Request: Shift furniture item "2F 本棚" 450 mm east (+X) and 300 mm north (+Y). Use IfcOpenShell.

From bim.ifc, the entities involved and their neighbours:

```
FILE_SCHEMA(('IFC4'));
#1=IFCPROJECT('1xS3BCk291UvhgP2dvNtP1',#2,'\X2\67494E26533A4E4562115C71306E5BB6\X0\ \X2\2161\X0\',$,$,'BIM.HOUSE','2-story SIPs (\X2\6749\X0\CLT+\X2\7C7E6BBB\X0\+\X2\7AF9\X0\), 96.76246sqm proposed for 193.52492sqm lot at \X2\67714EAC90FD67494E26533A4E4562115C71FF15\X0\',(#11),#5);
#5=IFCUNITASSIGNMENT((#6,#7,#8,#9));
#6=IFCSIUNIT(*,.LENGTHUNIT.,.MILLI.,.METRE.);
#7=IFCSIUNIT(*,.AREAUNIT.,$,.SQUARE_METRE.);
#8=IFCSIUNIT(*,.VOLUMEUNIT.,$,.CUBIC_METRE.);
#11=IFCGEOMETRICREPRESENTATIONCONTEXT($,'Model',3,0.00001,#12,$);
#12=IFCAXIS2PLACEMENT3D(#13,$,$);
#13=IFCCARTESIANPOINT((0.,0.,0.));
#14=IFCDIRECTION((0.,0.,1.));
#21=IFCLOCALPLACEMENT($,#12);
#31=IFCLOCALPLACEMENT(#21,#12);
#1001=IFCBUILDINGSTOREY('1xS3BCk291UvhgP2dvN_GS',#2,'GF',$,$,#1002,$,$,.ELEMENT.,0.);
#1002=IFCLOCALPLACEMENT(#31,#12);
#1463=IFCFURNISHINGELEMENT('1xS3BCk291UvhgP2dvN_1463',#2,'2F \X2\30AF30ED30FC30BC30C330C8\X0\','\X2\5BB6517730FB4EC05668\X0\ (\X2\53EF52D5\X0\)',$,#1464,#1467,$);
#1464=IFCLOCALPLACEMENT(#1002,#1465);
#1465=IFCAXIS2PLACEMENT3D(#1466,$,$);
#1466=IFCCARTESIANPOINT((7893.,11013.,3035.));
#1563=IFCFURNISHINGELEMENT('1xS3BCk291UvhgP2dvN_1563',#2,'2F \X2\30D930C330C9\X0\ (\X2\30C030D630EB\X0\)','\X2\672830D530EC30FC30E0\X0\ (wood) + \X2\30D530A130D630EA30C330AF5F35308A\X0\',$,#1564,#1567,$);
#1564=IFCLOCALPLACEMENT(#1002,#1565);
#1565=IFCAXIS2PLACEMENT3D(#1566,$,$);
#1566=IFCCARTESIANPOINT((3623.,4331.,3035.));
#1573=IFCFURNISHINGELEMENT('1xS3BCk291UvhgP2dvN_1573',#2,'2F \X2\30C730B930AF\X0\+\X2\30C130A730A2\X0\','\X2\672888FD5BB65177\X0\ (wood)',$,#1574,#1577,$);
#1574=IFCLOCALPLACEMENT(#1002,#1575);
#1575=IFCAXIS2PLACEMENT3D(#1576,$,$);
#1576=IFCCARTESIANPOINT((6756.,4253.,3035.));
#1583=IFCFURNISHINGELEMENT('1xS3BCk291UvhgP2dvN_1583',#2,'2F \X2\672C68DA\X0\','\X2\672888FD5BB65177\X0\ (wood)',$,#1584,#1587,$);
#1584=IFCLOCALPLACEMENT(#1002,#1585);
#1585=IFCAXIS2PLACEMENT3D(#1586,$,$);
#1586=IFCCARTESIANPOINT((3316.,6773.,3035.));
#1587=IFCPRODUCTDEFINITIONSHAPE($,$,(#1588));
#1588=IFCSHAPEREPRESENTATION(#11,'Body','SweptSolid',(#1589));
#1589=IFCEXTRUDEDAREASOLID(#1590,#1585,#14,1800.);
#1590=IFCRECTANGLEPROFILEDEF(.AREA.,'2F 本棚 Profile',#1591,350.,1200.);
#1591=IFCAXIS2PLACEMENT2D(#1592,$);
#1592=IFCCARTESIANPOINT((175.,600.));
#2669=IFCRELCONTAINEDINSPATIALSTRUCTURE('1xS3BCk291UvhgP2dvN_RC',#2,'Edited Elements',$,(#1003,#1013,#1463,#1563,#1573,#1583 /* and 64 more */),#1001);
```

```python
import ifcopenshell
import ifcopenshell.api.geometry
import ifcopenshell.util.placement
import ifcopenshell.util.unit

model = ifcopenshell.open("bim.ifc")
unit_scale = ifcopenshell.util.unit.calculate_unit_scale(model)

item = model.by_id(1583)
matrix = ifcopenshell.util.placement.get_local_placement(item.ObjectPlacement)
matrix[0, 3] += 0.45 / unit_scale
matrix[1, 3] += 0.3 / unit_scale
ifcopenshell.api.geometry.edit_object_placement(model, product=item, matrix=matrix, is_si=False)

print(ifcopenshell.util.placement.get_local_placement(item.ObjectPlacement).round(3) + 0.0)

model.write("bim_updated.ifc")
```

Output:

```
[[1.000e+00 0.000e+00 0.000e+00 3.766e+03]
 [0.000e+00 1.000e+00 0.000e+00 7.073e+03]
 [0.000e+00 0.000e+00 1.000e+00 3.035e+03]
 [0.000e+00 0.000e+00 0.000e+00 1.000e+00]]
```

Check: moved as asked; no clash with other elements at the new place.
